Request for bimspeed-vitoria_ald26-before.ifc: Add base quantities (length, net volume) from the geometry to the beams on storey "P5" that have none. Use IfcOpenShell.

First a look at what the model holds.

```python
import ifcopenshell
import ifcopenshell.util.element
import ifcopenshell.util.unit

model = ifcopenshell.open("bimspeed-vitoria_ald26-before.ifc")
print(model.schema)
for unit_type in ("LENGTHUNIT", "AREAUNIT", "VOLUMEUNIT"):
    print(unit_type, ifcopenshell.util.unit.calculate_unit_scale(model, unit_type))
storey = next(s for s in model.by_type("IfcBuildingStorey") if s.Name == "P5")
beams = [e for e in ifcopenshell.util.element.get_decomposition(storey) if e.is_a("IfcBeam")]
for e in sorted(beams, key=lambda e: e.id()):
    print(e.id(), e.is_a(), e.Name, list(ifcopenshell.util.element.get_psets(e, qtos_only=True)), sep=" | ")
```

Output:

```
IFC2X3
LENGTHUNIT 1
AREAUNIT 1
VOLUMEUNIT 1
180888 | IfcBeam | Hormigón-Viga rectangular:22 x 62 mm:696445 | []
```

```python
import ifcopenshell
import ifcopenshell.api.pset
import ifcopenshell.geom
import ifcopenshell.util.element
import ifcopenshell.util.shape
import ifcopenshell.util.unit

model = ifcopenshell.open("bimspeed-vitoria_ald26-before.ifc")
unit_scale = ifcopenshell.util.unit.calculate_unit_scale(model)
volume_scale = ifcopenshell.util.unit.calculate_unit_scale(model, "VOLUMEUNIT")
settings = ifcopenshell.geom.settings()

storey = next(s for s in model.by_type("IfcBuildingStorey") if s.Name == "P5")
beams = [e for e in ifcopenshell.util.element.get_decomposition(storey) if e.is_a("IfcBeam")]

for e in sorted(beams, key=lambda e: e.id()):
    if ifcopenshell.util.element.get_psets(e, qtos_only=True, should_inherit=False):
        continue
    # Geometry comes back in metres, in the element's own axes.
    shape = ifcopenshell.geom.create_shape(settings, e)
    values = {
        "Length": ifcopenshell.util.shape.get_max_xyz(shape.geometry) / unit_scale,
        "NetVolume": ifcopenshell.util.shape.get_volume(shape.geometry) / volume_scale,
    }
    qto = ifcopenshell.api.pset.add_qto(model, product=e, name="BaseQuantities")
    ifcopenshell.api.pset.edit_qto(model, qto=qto, properties=values)
    print(e.id(), {k: round(v, 3) for k, v in values.items()})

model.write("bimspeed-vitoria_ald26-before-out.ifc")
```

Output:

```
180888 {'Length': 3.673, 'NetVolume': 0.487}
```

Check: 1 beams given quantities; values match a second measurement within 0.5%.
